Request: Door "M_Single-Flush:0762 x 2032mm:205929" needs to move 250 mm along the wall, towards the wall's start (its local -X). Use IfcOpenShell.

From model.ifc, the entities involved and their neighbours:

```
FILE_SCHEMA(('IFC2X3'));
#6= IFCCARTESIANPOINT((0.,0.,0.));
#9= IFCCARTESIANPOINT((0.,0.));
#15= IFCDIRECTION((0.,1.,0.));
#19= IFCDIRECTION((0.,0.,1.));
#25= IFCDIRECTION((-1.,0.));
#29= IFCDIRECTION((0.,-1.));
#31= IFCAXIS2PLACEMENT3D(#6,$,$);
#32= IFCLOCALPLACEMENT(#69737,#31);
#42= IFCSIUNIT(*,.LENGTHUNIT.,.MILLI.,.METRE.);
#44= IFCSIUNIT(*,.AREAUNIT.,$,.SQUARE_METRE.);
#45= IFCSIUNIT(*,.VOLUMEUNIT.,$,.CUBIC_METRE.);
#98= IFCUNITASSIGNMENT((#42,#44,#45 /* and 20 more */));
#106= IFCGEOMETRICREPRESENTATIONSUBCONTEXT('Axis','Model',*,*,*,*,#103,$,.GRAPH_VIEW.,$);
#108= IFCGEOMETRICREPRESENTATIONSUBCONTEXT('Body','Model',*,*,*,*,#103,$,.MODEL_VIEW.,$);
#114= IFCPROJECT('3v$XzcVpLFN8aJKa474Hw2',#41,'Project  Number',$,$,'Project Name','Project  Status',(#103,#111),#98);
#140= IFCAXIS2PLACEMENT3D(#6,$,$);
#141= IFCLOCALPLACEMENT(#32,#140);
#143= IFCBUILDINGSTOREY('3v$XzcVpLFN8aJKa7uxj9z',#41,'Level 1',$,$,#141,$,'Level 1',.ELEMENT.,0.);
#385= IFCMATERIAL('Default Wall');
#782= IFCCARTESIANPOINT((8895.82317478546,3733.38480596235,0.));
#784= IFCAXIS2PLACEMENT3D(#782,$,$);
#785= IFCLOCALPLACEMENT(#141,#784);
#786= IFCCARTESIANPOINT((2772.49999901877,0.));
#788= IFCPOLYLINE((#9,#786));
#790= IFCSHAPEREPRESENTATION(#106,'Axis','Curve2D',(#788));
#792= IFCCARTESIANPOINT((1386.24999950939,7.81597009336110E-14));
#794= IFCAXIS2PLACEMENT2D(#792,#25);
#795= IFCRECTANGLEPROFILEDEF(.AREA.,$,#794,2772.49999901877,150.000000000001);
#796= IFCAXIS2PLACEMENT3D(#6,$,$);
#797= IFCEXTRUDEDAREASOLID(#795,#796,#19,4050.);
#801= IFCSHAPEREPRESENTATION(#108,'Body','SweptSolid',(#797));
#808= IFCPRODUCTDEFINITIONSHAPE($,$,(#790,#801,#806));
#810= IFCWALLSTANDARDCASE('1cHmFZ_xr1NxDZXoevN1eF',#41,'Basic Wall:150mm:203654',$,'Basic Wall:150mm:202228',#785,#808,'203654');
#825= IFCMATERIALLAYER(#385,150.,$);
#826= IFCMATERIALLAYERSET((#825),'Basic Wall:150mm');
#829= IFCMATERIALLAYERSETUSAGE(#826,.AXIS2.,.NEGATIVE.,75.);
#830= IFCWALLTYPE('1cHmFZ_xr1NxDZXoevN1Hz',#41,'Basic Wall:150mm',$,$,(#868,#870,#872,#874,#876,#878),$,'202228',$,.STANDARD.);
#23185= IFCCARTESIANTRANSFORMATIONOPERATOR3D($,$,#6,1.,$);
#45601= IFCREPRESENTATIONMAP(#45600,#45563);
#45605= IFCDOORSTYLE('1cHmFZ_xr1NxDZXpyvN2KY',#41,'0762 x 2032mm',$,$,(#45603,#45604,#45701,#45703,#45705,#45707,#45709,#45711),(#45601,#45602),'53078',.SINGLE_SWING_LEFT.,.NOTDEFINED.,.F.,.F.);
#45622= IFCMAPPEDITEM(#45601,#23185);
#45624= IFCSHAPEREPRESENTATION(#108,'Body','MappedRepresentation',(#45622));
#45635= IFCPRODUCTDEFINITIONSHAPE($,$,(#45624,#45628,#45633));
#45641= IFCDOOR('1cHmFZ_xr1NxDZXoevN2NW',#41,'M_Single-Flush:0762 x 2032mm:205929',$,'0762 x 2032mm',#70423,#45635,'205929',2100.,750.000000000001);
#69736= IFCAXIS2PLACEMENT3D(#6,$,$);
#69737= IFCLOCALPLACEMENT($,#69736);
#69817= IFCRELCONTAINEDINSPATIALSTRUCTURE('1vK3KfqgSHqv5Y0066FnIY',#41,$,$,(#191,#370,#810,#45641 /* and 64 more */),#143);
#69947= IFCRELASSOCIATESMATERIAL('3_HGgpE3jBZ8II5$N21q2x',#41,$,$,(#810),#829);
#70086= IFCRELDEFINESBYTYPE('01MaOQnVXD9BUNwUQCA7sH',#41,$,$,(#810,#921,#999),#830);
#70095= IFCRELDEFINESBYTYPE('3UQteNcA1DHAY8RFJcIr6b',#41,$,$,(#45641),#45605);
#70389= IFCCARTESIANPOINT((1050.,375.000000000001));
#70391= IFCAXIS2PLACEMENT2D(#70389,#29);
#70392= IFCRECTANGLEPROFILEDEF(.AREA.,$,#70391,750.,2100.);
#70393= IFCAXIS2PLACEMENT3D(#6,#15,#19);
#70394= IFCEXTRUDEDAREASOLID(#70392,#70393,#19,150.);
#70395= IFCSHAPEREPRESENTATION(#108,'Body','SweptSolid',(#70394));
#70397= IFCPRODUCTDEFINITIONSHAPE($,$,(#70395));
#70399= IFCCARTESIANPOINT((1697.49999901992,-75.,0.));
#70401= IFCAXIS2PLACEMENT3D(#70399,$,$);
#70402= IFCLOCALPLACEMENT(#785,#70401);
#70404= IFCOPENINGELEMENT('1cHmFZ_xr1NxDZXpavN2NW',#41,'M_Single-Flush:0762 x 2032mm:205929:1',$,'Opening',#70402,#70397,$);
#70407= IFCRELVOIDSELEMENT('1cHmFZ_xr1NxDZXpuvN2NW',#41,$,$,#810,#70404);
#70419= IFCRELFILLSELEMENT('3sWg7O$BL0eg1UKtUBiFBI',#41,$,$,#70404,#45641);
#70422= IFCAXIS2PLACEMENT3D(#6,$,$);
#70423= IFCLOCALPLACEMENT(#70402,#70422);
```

```python
import ifcopenshell
import ifcopenshell.api.geometry
import ifcopenshell.util.placement
import ifcopenshell.util.unit

model = ifcopenshell.open("model.ifc")
unit_scale = ifcopenshell.util.unit.calculate_unit_scale(model)

door = model.by_id(45641)
opening = door.FillsVoids[0].RelatingOpeningElement
wall = opening.VoidsElements[0].RelatingBuildingElement

wall_matrix = ifcopenshell.util.placement.get_local_placement(wall.ObjectPlacement)
shift = wall_matrix[:3, 0] * -0.25 / unit_scale
before = ifcopenshell.util.placement.get_local_placement(door.ObjectPlacement)[:3, 3].copy()

# The door is placed relative to its opening, so it follows when the opening moves.
matrix = ifcopenshell.util.placement.get_local_placement(opening.ObjectPlacement)
matrix[:3, 3] += shift
ifcopenshell.api.geometry.edit_object_placement(
    model, product=opening, matrix=matrix, is_si=False, should_transform_children=True
)

after = ifcopenshell.util.placement.get_local_placement(door.ObjectPlacement)[:3, 3]
print("door moved by", (after - before).round(3) + 0.0)

model.write("model_updated.ifc")
```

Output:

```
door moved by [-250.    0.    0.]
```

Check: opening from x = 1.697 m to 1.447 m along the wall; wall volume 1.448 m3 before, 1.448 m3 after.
